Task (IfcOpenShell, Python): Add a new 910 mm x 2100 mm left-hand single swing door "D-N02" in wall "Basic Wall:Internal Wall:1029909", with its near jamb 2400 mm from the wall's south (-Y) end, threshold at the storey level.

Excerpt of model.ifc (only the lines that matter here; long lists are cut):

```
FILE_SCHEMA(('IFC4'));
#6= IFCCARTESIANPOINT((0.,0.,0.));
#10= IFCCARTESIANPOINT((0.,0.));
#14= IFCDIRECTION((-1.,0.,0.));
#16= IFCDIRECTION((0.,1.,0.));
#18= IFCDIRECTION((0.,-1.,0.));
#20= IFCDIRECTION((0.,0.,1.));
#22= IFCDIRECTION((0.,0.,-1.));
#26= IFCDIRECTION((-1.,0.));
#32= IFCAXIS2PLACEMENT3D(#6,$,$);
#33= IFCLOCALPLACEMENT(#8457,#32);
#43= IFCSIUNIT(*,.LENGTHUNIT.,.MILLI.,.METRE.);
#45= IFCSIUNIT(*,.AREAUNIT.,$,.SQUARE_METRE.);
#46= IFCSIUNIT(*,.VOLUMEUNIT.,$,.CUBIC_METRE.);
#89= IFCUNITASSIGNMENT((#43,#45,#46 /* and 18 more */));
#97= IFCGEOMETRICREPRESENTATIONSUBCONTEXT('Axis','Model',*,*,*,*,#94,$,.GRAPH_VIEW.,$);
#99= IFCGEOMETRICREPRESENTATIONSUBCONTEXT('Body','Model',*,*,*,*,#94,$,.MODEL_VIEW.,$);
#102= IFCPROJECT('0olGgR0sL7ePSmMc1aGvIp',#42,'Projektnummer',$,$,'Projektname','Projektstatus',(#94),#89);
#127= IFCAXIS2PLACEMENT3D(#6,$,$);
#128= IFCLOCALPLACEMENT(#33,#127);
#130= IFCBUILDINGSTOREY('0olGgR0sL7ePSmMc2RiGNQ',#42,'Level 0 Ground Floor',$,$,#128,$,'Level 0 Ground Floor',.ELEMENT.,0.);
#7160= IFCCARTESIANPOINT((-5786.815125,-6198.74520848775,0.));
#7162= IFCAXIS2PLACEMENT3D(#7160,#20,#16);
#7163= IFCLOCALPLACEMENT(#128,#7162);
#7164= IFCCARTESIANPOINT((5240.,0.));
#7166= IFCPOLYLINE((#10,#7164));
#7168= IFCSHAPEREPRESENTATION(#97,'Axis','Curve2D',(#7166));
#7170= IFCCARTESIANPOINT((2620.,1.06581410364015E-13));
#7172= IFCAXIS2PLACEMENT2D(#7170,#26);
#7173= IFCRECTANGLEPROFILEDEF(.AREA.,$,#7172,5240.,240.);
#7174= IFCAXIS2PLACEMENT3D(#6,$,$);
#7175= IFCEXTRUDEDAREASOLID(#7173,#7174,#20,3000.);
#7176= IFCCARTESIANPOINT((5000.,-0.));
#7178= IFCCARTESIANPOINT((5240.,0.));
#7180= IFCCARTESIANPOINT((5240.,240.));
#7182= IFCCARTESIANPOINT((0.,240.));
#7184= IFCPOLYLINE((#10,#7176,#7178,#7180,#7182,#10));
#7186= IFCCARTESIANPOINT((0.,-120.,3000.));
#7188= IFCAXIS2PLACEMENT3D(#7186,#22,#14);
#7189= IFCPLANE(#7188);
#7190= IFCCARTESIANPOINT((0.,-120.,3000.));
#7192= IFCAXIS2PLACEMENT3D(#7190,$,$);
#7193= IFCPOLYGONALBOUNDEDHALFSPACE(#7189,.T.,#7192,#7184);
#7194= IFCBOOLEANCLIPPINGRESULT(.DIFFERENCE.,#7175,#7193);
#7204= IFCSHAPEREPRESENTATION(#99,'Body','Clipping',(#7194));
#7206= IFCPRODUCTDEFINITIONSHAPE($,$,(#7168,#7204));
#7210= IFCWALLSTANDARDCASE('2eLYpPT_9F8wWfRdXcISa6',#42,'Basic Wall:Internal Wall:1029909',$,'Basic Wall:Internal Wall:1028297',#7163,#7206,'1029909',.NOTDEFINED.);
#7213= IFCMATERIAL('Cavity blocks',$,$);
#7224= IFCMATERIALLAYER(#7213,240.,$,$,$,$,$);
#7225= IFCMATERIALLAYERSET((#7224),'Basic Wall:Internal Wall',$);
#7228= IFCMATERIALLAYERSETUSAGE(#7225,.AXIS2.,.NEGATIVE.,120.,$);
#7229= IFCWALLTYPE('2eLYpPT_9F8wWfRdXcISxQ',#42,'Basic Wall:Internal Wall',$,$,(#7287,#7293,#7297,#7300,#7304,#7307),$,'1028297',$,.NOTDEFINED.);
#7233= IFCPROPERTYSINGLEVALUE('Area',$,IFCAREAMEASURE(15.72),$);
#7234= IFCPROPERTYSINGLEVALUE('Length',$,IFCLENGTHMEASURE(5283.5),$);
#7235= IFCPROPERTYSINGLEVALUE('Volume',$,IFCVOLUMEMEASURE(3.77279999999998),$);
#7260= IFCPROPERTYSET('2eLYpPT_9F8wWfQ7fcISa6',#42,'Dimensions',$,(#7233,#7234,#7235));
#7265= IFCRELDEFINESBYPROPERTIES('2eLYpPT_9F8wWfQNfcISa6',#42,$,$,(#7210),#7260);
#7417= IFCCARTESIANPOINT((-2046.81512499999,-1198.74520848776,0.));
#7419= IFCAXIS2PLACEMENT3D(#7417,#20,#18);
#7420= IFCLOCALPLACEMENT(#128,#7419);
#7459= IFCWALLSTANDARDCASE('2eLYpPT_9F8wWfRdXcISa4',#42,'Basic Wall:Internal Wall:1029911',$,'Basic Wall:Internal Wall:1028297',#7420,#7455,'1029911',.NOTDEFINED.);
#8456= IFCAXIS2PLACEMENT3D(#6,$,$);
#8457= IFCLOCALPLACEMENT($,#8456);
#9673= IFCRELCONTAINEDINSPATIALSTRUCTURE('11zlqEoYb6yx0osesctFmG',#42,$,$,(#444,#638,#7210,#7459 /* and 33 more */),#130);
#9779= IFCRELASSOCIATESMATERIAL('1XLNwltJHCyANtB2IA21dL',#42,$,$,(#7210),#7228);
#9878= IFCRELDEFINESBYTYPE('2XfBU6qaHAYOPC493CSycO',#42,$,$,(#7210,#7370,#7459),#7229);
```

```python
import numpy as np
import ifcopenshell
import ifcopenshell.api.feature
import ifcopenshell.api.geometry
import ifcopenshell.api.pset
import ifcopenshell.api.root
import ifcopenshell.api.spatial
import ifcopenshell.geom
import ifcopenshell.util.element
import ifcopenshell.util.placement
import ifcopenshell.util.representation
import ifcopenshell.util.shape
import ifcopenshell.util.unit

model = ifcopenshell.open("model.ifc")
unit_scale = ifcopenshell.util.unit.calculate_unit_scale(model)
area_scale = ifcopenshell.util.unit.calculate_unit_scale(model, "AREAUNIT")
volume_scale = ifcopenshell.util.unit.calculate_unit_scale(model, "VOLUMEUNIT")
settings = ifcopenshell.geom.settings()


def volume(element):
    """Net volume in cubic metres, openings subtracted."""
    shape = ifcopenshell.geom.create_shape(settings, element)
    return ifcopenshell.util.shape.get_volume(shape.geometry)


wall = model.by_guid("2eLYpPT_9F8wWfRdXcISa6")
storey = ifcopenshell.util.element.get_container(wall, ifc_class="IfcBuildingStorey")
context = ifcopenshell.util.representation.get_context(model, "Model", "Body", "MODEL_VIEW")
before = volume(wall)

width, height, from_end, sill = 0.91, 2.1, 2.4, 0.0  # metres

# The wall runs along its own X axis, and the end named is its -X end.
wall_shape = ifcopenshell.geom.create_shape(settings, wall)
x, y, z = ifcopenshell.util.shape.get_vertices(wall_shape.geometry).T
start = x.min() + from_end
face, thickness = float(y.min()), float(y.max() - y.min())
wall_matrix = ifcopenshell.util.placement.get_local_placement(wall.ObjectPlacement)
level = ifcopenshell.util.placement.get_local_placement(storey.ObjectPlacement)[2, 3]


def in_wall(x, y):
    """Placement at x, y metres in the wall's axes, at sill height."""
    matrix = wall_matrix.copy()
    matrix[:, 3] = wall_matrix @ np.array([x / unit_scale, y / unit_scale, 0.0, 1.0])
    matrix[2, 3] = level + sill / unit_scale
    return matrix


# Opening: a box that overshoots both wall faces by 50 mm.
opening = ifcopenshell.api.root.create_entity(model, ifc_class="IfcOpeningElement", predefined_type="OPENING")
box = ifcopenshell.api.geometry.add_wall_representation(
    model, context=context, length=width, height=height, thickness=thickness + 0.1
)
ifcopenshell.api.geometry.assign_representation(model, product=opening, representation=box)
ifcopenshell.api.geometry.edit_object_placement(model, product=opening, matrix=in_wall(start, face - 0.05), is_si=False)
ifcopenshell.api.feature.add_feature(model, feature=opening, element=wall)

door = ifcopenshell.api.root.create_entity(model, ifc_class="IfcDoor", name="D-N02", predefined_type="DOOR")
door.OverallWidth, door.OverallHeight = width / unit_scale, height / unit_scale
door.OperationType = "SINGLE_SWING_LEFT"
body = ifcopenshell.api.geometry.add_door_representation(
    model,
    context=context,
    overall_width=door.OverallWidth,
    overall_height=door.OverallHeight,
    operation_type="SINGLE_SWING_LEFT",
    lining_properties={"LiningDepth": thickness / unit_scale, "ThresholdDepth": thickness / unit_scale},
)
ifcopenshell.api.geometry.assign_representation(model, product=door, representation=body)
ifcopenshell.api.spatial.assign_container(model, products=[door], relating_structure=storey)
ifcopenshell.api.feature.add_filling(model, opening=opening, element=door)

# The lining spans the wall, so the door starts at the wall face.
ifcopenshell.api.geometry.edit_object_placement(model, product=door, matrix=in_wall(start, face), is_si=False)

after = volume(wall)

# Update the wall's stored quantities.
pset = model.by_id(ifcopenshell.util.element.get_pset(wall, "Dimensions", should_inherit=False)["id"])
ifcopenshell.api.pset.edit_pset(model, pset=pset, properties={
    "Area": model.create_entity("IfcAreaMeasure", after / thickness / area_scale),
    "Volume": model.create_entity("IfcVolumeMeasure", after / volume_scale),
})

print(f"wall volume {before:.3f} -> {after:.3f} m3")

model.write("model_v2.ifc")
```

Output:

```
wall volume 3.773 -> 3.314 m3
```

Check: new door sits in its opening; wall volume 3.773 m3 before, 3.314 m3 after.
